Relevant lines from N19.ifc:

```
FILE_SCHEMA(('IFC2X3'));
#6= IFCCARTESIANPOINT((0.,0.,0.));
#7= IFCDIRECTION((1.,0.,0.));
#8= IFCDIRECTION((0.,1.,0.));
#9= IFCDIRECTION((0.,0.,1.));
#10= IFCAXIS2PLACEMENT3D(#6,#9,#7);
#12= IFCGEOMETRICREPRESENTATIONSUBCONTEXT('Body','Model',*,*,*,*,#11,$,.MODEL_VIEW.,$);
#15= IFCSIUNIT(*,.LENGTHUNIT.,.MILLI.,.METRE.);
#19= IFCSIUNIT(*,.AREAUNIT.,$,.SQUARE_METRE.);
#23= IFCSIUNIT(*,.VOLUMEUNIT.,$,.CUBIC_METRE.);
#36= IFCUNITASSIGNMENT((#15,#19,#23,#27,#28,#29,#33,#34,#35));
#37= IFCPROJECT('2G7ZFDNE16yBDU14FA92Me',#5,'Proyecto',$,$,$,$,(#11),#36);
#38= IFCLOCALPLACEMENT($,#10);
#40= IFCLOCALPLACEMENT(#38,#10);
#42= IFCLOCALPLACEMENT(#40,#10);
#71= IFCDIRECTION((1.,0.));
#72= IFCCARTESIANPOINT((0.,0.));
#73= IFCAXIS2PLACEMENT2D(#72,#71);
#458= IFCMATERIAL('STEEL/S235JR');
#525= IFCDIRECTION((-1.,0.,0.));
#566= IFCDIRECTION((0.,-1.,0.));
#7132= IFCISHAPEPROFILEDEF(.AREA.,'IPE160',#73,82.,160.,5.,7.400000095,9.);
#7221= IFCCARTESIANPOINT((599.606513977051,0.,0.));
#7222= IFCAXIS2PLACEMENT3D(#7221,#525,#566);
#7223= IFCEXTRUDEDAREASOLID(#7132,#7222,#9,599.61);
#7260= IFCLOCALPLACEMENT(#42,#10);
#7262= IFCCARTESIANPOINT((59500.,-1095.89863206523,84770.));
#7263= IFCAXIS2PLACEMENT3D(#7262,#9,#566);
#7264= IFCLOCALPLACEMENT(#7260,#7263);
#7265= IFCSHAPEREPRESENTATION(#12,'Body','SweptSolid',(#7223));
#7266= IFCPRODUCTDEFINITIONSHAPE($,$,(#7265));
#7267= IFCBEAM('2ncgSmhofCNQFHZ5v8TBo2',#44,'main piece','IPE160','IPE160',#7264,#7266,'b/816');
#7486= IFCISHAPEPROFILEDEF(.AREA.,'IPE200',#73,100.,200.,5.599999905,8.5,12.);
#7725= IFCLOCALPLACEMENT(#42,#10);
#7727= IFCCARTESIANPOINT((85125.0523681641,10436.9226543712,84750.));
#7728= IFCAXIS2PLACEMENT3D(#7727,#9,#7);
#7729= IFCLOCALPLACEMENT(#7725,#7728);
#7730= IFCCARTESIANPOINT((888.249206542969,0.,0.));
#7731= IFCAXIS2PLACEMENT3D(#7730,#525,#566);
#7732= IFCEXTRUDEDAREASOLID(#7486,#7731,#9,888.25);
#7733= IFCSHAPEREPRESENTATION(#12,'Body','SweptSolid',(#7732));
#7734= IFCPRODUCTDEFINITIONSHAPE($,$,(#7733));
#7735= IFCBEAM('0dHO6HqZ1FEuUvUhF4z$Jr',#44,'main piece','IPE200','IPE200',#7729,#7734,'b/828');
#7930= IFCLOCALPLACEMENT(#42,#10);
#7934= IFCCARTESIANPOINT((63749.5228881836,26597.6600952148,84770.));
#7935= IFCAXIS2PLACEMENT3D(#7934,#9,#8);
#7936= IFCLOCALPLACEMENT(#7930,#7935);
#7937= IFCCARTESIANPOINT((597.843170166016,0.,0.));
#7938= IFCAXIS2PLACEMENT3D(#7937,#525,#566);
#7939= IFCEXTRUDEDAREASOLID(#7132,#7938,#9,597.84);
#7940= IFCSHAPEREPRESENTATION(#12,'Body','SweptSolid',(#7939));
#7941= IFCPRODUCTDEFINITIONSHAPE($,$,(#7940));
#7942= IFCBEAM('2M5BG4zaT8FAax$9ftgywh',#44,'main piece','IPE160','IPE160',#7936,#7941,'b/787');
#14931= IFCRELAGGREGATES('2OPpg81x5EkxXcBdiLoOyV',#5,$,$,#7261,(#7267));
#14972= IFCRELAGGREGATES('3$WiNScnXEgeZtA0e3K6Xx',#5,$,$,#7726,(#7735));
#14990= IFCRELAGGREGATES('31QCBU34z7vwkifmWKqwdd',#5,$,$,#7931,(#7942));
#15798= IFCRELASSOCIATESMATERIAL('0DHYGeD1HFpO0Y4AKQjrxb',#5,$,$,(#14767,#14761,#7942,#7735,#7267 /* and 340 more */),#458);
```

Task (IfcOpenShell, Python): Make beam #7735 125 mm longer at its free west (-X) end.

```python
import ifcopenshell
import ifcopenshell.util.representation

model = ifcopenshell.open("N19.ifc")

member = model.by_guid("0dHO6HqZ1FEuUvUhF4z$Jr")
change = 125.0

# The extrusion runs towards the end named, so only its depth changes.
body = ifcopenshell.util.representation.get_representation(member, "Model", "Body")
solid = body.Items[0]
old_length = solid.Depth
solid.Depth += change

print(f"length {old_length:g} -> {solid.Depth:g}")

model.write("N19-out.ifc")
```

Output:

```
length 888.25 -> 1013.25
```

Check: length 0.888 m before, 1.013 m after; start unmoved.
